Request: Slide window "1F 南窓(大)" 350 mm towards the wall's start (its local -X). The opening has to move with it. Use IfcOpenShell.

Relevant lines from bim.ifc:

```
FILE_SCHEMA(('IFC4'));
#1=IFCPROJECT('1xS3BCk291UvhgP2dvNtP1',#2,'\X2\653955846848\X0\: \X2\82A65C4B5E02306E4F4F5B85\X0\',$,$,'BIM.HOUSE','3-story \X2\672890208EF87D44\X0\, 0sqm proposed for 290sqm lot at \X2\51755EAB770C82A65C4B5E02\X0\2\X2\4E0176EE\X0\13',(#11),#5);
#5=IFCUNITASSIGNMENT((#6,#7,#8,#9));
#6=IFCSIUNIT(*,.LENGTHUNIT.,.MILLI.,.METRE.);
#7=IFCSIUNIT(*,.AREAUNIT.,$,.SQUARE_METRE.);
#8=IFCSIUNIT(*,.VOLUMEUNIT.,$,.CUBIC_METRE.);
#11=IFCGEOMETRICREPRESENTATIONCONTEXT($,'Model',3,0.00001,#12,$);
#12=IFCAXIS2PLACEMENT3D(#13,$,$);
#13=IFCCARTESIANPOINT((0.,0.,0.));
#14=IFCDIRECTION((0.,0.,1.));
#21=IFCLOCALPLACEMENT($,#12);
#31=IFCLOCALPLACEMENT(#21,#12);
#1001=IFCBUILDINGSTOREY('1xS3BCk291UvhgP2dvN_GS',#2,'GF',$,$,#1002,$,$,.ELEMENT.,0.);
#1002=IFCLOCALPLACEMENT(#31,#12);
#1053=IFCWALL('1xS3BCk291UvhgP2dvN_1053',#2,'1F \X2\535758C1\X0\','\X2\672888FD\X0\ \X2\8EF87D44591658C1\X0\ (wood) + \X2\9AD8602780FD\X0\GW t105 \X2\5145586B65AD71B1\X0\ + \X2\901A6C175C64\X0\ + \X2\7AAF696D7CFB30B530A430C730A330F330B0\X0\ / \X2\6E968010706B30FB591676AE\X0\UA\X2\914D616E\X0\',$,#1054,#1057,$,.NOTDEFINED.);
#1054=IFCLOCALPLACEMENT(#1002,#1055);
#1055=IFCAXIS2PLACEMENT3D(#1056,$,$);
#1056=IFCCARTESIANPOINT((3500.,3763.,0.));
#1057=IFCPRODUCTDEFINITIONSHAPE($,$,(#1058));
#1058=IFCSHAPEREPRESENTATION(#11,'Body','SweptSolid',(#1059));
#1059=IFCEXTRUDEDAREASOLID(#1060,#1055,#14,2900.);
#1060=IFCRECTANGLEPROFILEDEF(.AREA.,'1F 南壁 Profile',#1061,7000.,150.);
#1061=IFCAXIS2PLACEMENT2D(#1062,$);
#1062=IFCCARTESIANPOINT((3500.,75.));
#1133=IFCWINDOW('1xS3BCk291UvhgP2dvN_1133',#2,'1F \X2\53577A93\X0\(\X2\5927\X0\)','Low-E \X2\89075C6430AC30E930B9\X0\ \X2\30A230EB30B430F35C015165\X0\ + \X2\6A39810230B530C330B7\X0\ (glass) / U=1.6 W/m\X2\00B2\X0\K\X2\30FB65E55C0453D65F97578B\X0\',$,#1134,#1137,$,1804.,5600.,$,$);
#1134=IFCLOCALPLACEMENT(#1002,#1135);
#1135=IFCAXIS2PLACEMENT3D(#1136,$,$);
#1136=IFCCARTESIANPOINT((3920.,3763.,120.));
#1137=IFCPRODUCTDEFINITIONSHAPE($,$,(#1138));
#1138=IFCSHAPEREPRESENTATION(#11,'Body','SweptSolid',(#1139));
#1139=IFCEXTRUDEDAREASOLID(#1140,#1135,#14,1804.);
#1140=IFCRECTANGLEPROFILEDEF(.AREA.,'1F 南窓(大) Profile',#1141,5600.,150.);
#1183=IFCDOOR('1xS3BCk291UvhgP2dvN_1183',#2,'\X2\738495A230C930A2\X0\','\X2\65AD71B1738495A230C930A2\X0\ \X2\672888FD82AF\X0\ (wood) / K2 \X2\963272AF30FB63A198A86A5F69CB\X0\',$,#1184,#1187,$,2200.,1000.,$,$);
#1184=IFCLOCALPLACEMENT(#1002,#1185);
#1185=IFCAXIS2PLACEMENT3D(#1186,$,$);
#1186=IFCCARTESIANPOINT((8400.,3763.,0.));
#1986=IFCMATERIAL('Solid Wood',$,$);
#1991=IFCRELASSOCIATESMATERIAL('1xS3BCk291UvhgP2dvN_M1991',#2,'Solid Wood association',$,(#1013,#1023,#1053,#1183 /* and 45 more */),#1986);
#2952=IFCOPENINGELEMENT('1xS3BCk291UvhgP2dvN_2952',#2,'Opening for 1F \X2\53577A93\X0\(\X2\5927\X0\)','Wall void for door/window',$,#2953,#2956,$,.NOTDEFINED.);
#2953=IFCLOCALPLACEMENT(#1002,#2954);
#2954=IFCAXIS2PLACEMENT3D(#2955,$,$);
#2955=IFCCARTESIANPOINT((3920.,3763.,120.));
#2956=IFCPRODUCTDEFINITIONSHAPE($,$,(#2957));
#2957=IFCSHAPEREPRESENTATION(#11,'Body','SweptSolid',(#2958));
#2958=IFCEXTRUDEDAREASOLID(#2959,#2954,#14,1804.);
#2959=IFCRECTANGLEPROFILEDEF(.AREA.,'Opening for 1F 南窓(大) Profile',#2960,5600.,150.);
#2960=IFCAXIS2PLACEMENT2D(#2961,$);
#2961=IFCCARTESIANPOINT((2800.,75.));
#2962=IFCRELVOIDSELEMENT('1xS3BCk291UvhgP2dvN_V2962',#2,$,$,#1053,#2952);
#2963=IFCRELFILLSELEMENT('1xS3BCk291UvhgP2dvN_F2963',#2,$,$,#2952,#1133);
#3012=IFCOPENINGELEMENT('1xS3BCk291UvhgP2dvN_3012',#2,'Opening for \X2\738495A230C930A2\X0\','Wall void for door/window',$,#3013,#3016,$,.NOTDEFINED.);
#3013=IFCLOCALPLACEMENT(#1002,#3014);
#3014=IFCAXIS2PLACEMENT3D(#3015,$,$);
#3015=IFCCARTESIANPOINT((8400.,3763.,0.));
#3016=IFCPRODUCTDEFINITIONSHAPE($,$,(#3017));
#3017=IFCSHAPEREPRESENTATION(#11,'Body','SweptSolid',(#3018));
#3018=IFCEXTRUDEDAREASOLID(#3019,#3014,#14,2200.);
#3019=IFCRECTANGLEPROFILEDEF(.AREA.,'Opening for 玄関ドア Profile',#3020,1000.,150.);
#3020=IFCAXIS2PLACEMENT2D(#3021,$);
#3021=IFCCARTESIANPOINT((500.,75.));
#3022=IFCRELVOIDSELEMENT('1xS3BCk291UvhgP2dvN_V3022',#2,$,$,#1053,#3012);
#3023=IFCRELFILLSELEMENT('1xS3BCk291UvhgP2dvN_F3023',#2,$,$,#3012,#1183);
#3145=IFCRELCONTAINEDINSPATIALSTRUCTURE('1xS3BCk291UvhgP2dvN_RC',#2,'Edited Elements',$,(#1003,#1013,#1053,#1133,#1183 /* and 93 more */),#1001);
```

```python
import ifcopenshell
import ifcopenshell.api.geometry
import ifcopenshell.util.placement
import ifcopenshell.util.unit

model = ifcopenshell.open("bim.ifc")
unit_scale = ifcopenshell.util.unit.calculate_unit_scale(model)

window = model.by_id(1133)
opening = window.FillsVoids[0].RelatingOpeningElement
wall = opening.VoidsElements[0].RelatingBuildingElement

wall_matrix = ifcopenshell.util.placement.get_local_placement(wall.ObjectPlacement)
shift = wall_matrix[:3, 0] * -0.35 / unit_scale
before = ifcopenshell.util.placement.get_local_placement(window.ObjectPlacement)[:3, 3].copy()

# The window is not placed relative to its opening, so move both.
for product in (opening, window):
    matrix = ifcopenshell.util.placement.get_local_placement(product.ObjectPlacement)
    matrix[:3, 3] += shift
    ifcopenshell.api.geometry.edit_object_placement(model, product=product, matrix=matrix, is_si=False)

after = ifcopenshell.util.placement.get_local_placement(window.ObjectPlacement)[:3, 3]
print("window moved by", (after - before).round(3) + 0.0)

model.write("bim-out.ifc")
```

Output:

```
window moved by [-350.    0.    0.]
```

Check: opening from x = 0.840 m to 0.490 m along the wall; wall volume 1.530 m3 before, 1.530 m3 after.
